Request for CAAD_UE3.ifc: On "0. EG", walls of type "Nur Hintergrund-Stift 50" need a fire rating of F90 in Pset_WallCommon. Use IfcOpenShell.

First a look at what the model holds.

```python
import ifcopenshell
import ifcopenshell.util.element

model = ifcopenshell.open("CAAD_UE3.ifc")
print(model.schema)
storey = next(s for s in model.by_type("IfcBuildingStorey") if s.Name == "0. EG")
walls = [e for e in ifcopenshell.util.element.get_decomposition(storey) if e.is_a("IfcWall")]
seen = {}
for e in walls:
    element_type = ifcopenshell.util.element.get_type(e)
    key = (element_type.Name if element_type != e and element_type else None, ifcopenshell.util.element.get_pset(e, "Pset_WallCommon", "FireRating"))
    seen[key] = seen.get(key, 0) + 1
for (name, value), count in sorted(seen.items(), key=str):
    print(count, "x", name, "|", value)
```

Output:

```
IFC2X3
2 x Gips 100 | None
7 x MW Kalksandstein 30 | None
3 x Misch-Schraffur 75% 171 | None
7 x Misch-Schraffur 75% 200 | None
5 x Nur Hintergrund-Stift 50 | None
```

```python
import ifcopenshell
import ifcopenshell.api.pset
import ifcopenshell.util.element

model = ifcopenshell.open("CAAD_UE3.ifc")

storey = next(s for s in model.by_type("IfcBuildingStorey") if s.Name == "0. EG")
walls = [e for e in ifcopenshell.util.element.get_decomposition(storey) if e.is_a("IfcWall")]

count = 0
for e in walls:
    element_type = ifcopenshell.util.element.get_type(e)
    if element_type in (None, e) or element_type.Name != "Nur Hintergrund-Stift 50":
        continue
    # add_pset returns the element's existing set when there is one.
    pset = ifcopenshell.api.pset.add_pset(model, product=e, name="Pset_WallCommon")
    ifcopenshell.api.pset.edit_pset(model, pset=pset, properties={"FireRating": "F90"})
    count += 1

print(count, "walls updated")

model.write("CAAD_UE3_rev.ifc")
```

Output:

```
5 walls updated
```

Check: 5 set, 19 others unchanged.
